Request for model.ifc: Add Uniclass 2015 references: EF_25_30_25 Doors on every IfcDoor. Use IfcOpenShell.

First a look at what the model holds.

```python
import ifcopenshell

model = ifcopenshell.open("model.ifc")
print(model.schema)
print("classifications:", [c.Name for c in model.by_type("IfcClassification")])
for ifc_class in ("IfcDoor", "IfcRoof", "IfcStair", "IfcWall", "IfcWindow"):
    print(ifc_class, len(model.by_type(ifc_class)))
```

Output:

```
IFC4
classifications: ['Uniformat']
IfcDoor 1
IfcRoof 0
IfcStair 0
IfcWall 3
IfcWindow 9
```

```python
import ifcopenshell
import ifcopenshell.api.classification

model = ifcopenshell.open("model.ifc")

system = ifcopenshell.api.classification.add_classification(model, classification="Uniclass 2015")

codes = {
    "IfcDoor": ("EF_25_30_25", "Doors"),
}
for ifc_class, (code, name) in codes.items():
    products = model.by_type(ifc_class)
    ifcopenshell.api.classification.add_reference(
        model, products=products, classification=system, identification=code, name=name
    )
    print(code, len(products))

model.write("model_rev.ifc")
```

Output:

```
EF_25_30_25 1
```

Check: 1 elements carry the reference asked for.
